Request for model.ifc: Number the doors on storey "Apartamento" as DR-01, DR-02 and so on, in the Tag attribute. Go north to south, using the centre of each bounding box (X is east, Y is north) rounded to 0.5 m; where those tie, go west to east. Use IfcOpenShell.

First a look at what the model holds.

```python
import ifcopenshell
import ifcopenshell.util.element
import ifcopenshell.util.placement

model = ifcopenshell.open("model.ifc")
print(model.schema)
storey = next(s for s in model.by_type("IfcBuildingStorey") if s.Name == "Apartamento")
doors = [e for e in ifcopenshell.util.element.get_decomposition(storey) if e.is_a("IfcDoor")]
for e in sorted(doors, key=lambda e: e.id()):
    origin = ifcopenshell.util.placement.get_local_placement(e.ObjectPlacement)[:3, 3]
    print(e.id(), e.Tag, e.Name, origin.round(2) + 0.0, sep=" | ")
```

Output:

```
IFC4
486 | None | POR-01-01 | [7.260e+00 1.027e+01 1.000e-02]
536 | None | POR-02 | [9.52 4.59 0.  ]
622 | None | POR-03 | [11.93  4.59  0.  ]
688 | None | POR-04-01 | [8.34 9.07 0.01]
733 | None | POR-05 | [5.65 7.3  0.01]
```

```python
import ifcopenshell
import ifcopenshell.geom
import ifcopenshell.util.element
import ifcopenshell.util.shape

model = ifcopenshell.open("model.ifc")
settings = ifcopenshell.geom.settings()
settings.set("use-world-coords", True)


def centre(element):
    shape = ifcopenshell.geom.create_shape(settings, element)
    return ifcopenshell.util.shape.get_bbox_centroid(shape.geometry)


storey = next(s for s in model.by_type("IfcBuildingStorey") if s.Name == "Apartamento")
doors = [e for e in ifcopenshell.util.element.get_decomposition(storey) if e.is_a("IfcDoor")]

# Insertion points can sit at a corner or the storey origin, so sort by the geometry (in metres).
centres = {e: centre(e) for e in doors}
doors.sort(key=lambda e: (-round(centres[e][1] / 0.5), centres[e][0]))

for i, e in enumerate(doors, start=1):
    number = f"DR-{i:02d}"
    e.Tag = number
    print(e.id(), number)

model.write("model_rev.ifc")
```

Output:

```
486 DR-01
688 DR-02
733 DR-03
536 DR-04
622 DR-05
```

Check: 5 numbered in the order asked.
